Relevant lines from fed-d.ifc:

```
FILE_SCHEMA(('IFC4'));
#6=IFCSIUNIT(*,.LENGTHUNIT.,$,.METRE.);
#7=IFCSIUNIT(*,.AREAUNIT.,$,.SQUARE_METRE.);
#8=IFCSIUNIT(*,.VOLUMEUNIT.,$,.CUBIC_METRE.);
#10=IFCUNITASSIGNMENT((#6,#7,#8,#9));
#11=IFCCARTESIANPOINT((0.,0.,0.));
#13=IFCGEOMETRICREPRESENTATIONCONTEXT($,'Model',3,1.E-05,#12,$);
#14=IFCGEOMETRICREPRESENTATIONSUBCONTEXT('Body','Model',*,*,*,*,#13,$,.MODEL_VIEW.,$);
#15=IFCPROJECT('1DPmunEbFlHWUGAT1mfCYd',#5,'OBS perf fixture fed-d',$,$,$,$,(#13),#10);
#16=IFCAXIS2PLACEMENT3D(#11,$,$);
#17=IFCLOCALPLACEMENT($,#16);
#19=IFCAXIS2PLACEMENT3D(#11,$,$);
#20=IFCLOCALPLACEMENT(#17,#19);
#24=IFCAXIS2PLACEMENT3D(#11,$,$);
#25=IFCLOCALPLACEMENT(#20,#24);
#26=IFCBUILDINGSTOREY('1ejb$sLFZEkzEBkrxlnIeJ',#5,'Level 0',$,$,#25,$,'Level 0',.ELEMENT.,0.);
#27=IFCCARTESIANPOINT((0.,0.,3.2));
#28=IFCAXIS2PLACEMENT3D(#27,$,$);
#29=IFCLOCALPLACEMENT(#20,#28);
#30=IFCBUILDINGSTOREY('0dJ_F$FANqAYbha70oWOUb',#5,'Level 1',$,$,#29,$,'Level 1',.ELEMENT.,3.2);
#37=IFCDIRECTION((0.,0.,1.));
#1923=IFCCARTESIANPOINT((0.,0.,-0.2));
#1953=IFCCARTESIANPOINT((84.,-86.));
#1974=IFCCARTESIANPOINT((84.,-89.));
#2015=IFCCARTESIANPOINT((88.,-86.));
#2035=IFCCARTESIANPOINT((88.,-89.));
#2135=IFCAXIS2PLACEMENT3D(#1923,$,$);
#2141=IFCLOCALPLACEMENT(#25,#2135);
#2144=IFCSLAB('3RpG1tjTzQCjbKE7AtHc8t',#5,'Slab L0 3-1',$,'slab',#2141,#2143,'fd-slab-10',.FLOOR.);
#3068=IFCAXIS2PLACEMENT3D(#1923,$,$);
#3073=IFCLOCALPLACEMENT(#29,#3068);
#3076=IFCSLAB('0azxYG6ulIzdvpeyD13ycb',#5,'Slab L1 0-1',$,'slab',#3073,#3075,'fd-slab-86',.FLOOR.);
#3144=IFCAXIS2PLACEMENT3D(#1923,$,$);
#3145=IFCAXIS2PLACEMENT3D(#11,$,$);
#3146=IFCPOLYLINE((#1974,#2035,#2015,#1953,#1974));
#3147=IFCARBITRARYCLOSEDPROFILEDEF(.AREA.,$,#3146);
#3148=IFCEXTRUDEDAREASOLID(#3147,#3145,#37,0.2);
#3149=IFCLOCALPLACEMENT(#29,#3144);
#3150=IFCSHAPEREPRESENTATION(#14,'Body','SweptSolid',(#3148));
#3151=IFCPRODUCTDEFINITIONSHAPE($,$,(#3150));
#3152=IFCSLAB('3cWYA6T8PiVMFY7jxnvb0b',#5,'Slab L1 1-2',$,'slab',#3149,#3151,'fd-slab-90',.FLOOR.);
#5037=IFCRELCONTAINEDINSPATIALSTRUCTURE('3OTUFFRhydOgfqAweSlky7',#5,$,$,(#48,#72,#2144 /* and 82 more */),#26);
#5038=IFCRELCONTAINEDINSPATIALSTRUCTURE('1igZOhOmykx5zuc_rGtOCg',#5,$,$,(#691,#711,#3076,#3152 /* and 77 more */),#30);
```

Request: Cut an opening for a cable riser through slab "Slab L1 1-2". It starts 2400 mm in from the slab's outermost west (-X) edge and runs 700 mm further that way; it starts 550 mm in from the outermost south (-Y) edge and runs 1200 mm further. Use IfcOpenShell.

```python
import numpy as np
import ifcopenshell
import ifcopenshell.api.feature
import ifcopenshell.api.geometry
import ifcopenshell.api.root
import ifcopenshell.geom
import ifcopenshell.util.placement
import ifcopenshell.util.representation
import ifcopenshell.util.shape
import ifcopenshell.util.unit

model = ifcopenshell.open("fed-d.ifc")
unit_scale = ifcopenshell.util.unit.calculate_unit_scale(model)
settings = ifcopenshell.geom.settings()


def volume(element):
    """Net volume in cubic metres, openings subtracted."""
    shape = ifcopenshell.geom.create_shape(settings, element)
    return ifcopenshell.util.shape.get_volume(shape.geometry)


slab = model.by_id(3152)
before = volume(slab)

# Extent in the slab's own axes, in metres. The edges named are its -X and -Y sides.
slab_shape = ifcopenshell.geom.create_shape(settings, slab)
vertices = ifcopenshell.util.shape.get_vertices(slab_shape.geometry)
x_min, y_min, bottom = vertices.min(axis=0)
top = vertices[:, 2].max()

opening = ifcopenshell.api.root.create_entity(model, ifc_class="IfcOpeningElement", name="Cable riser opening", predefined_type="OPENING")
context = ifcopenshell.util.representation.get_context(model, "Model", "Body", "MODEL_VIEW")
width, depth = 0.7, 1.2
outline = [(0.0, 0.0), (width, 0.0), (width, depth), (0.0, depth), (0.0, 0.0)]
# Overshoot both faces by 50 mm so the cut is clean.
shape = ifcopenshell.api.geometry.add_slab_representation(
    model, context=context, depth=top - bottom + 0.1, polyline=outline
)
ifcopenshell.api.geometry.assign_representation(model, product=opening, representation=shape)

matrix = ifcopenshell.util.placement.get_local_placement(slab.ObjectPlacement)
matrix[:, 3] = matrix @ np.append(np.array([x_min + 2.4, y_min + 0.55, bottom - 0.05]) / unit_scale, 1.0)
ifcopenshell.api.geometry.edit_object_placement(model, product=opening, matrix=matrix, is_si=False)
ifcopenshell.api.feature.add_feature(model, feature=opening, element=slab)

after = volume(slab)

print(f"slab volume {before:.3f} -> {after:.3f} m3")

model.write("fed-d_v2.ifc")
```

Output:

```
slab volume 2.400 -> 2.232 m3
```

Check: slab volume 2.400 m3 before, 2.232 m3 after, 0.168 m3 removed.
